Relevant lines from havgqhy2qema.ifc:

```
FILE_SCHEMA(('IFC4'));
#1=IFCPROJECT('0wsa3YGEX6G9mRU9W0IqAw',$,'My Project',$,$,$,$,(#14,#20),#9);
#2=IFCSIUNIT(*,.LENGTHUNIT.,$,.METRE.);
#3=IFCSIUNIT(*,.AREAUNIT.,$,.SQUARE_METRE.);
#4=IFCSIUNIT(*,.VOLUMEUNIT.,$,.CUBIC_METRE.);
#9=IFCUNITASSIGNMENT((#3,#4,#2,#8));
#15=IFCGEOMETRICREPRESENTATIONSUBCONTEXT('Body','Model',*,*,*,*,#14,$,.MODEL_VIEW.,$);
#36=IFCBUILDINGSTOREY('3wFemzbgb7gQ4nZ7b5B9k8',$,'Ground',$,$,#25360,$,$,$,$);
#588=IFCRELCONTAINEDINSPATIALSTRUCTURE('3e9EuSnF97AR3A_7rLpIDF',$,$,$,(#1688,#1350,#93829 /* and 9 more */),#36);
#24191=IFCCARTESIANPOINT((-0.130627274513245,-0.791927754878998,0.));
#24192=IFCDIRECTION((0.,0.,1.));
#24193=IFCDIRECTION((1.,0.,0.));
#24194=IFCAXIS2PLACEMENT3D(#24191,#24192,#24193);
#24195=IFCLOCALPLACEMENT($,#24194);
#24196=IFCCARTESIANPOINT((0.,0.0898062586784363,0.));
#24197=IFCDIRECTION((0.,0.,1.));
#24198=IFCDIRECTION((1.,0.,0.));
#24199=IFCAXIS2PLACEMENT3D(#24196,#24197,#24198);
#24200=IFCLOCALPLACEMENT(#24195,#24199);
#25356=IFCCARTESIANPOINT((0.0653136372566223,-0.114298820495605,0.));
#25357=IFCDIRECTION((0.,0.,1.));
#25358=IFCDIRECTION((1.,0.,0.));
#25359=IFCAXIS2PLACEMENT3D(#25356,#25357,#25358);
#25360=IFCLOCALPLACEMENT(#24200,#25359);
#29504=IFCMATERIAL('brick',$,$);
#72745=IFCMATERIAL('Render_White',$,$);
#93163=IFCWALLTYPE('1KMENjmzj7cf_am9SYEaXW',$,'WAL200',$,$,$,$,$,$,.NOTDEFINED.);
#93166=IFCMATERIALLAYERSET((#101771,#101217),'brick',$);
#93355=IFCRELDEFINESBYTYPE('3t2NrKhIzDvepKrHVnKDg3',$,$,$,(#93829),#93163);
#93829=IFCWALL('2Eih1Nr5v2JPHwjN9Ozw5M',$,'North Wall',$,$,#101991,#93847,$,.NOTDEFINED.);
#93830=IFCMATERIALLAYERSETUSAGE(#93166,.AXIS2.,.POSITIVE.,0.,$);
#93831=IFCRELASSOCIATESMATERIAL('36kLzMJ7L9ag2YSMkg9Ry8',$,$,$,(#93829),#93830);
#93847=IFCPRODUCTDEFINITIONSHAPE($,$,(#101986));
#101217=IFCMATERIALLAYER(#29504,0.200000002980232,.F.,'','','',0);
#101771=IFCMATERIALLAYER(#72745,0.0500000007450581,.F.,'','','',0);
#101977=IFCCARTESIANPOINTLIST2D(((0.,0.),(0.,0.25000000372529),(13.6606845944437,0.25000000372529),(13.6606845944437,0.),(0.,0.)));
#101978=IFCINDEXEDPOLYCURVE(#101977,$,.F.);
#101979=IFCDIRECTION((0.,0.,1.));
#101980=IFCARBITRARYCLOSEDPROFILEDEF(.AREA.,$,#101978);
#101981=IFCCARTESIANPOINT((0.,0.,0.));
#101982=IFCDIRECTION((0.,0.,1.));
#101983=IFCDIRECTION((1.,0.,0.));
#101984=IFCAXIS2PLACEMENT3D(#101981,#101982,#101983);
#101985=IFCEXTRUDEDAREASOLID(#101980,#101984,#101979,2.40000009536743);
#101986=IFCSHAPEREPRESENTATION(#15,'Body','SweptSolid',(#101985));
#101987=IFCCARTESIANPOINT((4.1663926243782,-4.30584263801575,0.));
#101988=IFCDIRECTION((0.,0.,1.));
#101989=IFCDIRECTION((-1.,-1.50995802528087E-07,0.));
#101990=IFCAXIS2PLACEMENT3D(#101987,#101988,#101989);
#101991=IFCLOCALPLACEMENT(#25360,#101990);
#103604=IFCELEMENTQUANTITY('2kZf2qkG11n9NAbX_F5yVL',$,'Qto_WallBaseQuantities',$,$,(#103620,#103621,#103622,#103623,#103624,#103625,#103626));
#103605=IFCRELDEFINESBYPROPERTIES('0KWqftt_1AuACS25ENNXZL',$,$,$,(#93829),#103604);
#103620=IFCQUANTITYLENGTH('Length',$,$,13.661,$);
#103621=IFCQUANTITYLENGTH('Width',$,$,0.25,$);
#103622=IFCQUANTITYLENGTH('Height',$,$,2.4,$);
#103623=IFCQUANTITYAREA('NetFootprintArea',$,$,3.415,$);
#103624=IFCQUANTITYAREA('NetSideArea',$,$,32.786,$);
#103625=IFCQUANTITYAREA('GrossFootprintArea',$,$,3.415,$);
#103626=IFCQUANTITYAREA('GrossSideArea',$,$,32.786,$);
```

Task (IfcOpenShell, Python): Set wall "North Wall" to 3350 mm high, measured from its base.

```python
import ifcopenshell
import ifcopenshell.api.pset
import ifcopenshell.geom
import ifcopenshell.util.element
import ifcopenshell.util.representation
import ifcopenshell.util.shape
import ifcopenshell.util.unit

model = ifcopenshell.open("havgqhy2qema.ifc")
unit_scale = ifcopenshell.util.unit.calculate_unit_scale(model)
area_scale = ifcopenshell.util.unit.calculate_unit_scale(model, "AREAUNIT")
settings = ifcopenshell.geom.settings()


def volume(element):
    """Net volume in cubic metres, openings subtracted."""
    shape = ifcopenshell.geom.create_shape(settings, element)
    return ifcopenshell.util.shape.get_volume(shape.geometry)


wall = model.by_id(93829)
before = volume(wall)

body = ifcopenshell.util.representation.get_representation(wall, "Model", "Body")
solid = body.Items[0]
old_height = solid.Depth
solid.Depth = 3.35
after = volume(wall)
thickness = 0.25  # wall thickness in metres

# Update the stored height, areas and volumes.
qto = model.by_id(ifcopenshell.util.element.get_pset(wall, "Qto_WallBaseQuantities", should_inherit=False)["id"])
ifcopenshell.api.pset.edit_qto(model, qto=qto, properties={
    "Height": solid.Depth,
    "NetSideArea": after / thickness / area_scale,
    "GrossSideArea": ifcopenshell.util.element.get_pset(wall, "Qto_WallBaseQuantities", "GrossSideArea") * solid.Depth / old_height,
})

print(f"height {old_height:g} -> {solid.Depth:g}, volume {before:.3f} -> {after:.3f} m3")

model.write("havgqhy2qema_rev.ifc")
```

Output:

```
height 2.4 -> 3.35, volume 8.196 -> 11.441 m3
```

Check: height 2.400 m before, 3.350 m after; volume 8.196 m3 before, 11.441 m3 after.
